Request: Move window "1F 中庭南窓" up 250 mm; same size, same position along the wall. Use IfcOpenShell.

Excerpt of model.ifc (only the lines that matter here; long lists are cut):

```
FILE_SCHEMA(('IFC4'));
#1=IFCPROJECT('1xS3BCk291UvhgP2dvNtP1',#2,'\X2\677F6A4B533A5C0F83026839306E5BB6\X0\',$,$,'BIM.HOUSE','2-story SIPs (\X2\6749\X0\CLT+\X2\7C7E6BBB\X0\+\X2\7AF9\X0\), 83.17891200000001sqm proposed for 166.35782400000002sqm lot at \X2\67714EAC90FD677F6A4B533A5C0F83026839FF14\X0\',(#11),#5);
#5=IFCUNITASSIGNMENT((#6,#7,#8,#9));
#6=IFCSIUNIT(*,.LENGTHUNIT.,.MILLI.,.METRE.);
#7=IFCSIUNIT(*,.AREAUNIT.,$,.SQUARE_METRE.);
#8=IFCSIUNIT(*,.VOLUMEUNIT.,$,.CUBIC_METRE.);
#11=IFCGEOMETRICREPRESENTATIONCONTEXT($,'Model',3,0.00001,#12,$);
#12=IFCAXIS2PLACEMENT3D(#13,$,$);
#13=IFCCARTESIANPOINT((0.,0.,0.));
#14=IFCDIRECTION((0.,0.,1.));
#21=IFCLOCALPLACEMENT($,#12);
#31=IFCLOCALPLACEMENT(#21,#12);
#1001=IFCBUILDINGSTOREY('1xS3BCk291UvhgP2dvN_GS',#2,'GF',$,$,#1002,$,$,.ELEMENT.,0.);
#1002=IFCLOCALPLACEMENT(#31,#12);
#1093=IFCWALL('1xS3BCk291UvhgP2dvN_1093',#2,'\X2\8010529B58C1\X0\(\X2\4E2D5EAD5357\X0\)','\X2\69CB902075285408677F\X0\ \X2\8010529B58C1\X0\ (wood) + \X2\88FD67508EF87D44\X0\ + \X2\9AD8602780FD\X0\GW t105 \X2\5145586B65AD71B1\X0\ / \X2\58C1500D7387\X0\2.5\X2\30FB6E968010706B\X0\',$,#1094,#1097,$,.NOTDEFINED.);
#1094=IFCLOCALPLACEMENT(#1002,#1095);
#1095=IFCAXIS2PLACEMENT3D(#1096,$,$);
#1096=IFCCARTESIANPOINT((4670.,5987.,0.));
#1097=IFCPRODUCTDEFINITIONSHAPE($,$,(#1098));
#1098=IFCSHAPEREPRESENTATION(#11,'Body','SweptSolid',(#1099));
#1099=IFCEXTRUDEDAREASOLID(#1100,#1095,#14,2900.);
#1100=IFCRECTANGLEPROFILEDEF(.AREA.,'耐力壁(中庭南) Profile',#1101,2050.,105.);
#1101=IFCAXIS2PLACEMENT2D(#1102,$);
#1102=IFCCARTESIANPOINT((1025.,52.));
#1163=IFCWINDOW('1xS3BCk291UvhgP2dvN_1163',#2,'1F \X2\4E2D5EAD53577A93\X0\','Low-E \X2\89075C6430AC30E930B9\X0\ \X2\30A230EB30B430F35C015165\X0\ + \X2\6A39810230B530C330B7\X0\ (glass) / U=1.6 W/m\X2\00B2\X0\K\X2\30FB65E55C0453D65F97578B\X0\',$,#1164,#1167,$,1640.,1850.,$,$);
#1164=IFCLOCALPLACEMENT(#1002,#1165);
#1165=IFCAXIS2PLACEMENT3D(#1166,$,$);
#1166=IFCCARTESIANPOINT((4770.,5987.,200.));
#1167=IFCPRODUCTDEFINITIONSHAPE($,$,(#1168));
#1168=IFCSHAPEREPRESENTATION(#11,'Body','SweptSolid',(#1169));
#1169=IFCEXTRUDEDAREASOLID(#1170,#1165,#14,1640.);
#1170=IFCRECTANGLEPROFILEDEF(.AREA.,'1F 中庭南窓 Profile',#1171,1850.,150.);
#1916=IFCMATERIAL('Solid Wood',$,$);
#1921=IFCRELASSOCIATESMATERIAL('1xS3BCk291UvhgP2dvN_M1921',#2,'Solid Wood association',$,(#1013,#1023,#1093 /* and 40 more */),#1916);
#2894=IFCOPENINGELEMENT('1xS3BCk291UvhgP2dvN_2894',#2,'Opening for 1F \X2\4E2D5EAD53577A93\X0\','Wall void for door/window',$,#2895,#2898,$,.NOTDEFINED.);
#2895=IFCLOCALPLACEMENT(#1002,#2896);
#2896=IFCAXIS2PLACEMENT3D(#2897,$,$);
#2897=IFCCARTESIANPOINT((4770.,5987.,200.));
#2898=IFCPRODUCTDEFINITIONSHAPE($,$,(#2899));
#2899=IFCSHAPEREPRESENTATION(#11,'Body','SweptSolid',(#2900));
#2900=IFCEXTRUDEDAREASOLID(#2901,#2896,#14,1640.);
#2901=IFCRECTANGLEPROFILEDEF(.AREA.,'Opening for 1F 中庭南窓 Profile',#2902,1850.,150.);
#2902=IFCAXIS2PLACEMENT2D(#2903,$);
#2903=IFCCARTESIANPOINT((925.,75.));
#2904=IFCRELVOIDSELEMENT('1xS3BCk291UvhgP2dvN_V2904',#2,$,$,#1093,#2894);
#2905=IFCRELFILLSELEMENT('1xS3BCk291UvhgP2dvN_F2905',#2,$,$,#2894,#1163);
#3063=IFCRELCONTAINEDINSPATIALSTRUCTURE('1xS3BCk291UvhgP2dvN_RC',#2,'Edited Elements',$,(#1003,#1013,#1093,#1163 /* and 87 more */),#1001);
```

```python
import numpy as np
import ifcopenshell
import ifcopenshell.api.geometry
import ifcopenshell.util.placement
import ifcopenshell.util.unit

model = ifcopenshell.open("model.ifc")
unit_scale = ifcopenshell.util.unit.calculate_unit_scale(model)

window = model.by_guid("1xS3BCk291UvhgP2dvN_1163")
opening = window.FillsVoids[0].RelatingOpeningElement
dz = 0.25 / unit_scale

shift = np.array([0.0, 0.0, dz])
# The window is not placed relative to its opening, so move both.
for product in (opening, window):
    matrix = ifcopenshell.util.placement.get_local_placement(product.ObjectPlacement)
    matrix[:3, 3] += shift
    ifcopenshell.api.geometry.edit_object_placement(model, product=product, matrix=matrix, is_si=False)

print(f"moved by {dz * unit_scale:+.3f} m")

model.write("model_edited.ifc")
```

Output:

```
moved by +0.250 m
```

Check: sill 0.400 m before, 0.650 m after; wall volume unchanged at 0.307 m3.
